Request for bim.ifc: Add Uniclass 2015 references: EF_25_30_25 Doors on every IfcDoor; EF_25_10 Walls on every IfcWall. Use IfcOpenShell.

First a look at what the model holds.

```python
import ifcopenshell

model = ifcopenshell.open("bim.ifc")
print(model.schema)
print("classifications:", [c.Name for c in model.by_type("IfcClassification")])
for ifc_class in ("IfcDoor", "IfcRoof", "IfcStair", "IfcWall", "IfcWindow"):
    print(ifc_class, len(model.by_type(ifc_class)))
```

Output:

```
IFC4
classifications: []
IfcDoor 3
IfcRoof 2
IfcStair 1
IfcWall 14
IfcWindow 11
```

```python
import ifcopenshell
import ifcopenshell.api.classification

model = ifcopenshell.open("bim.ifc")

system = ifcopenshell.api.classification.add_classification(model, classification="Uniclass 2015")

codes = {
    "IfcDoor": ("EF_25_30_25", "Doors"),
    "IfcWall": ("EF_25_10", "Walls"),
}
for ifc_class, (code, name) in codes.items():
    products = model.by_type(ifc_class)
    ifcopenshell.api.classification.add_reference(
        model, products=products, classification=system, identification=code, name=name
    )
    print(code, len(products))

model.write("bim_edited.ifc")
```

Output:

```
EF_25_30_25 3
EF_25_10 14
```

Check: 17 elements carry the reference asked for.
